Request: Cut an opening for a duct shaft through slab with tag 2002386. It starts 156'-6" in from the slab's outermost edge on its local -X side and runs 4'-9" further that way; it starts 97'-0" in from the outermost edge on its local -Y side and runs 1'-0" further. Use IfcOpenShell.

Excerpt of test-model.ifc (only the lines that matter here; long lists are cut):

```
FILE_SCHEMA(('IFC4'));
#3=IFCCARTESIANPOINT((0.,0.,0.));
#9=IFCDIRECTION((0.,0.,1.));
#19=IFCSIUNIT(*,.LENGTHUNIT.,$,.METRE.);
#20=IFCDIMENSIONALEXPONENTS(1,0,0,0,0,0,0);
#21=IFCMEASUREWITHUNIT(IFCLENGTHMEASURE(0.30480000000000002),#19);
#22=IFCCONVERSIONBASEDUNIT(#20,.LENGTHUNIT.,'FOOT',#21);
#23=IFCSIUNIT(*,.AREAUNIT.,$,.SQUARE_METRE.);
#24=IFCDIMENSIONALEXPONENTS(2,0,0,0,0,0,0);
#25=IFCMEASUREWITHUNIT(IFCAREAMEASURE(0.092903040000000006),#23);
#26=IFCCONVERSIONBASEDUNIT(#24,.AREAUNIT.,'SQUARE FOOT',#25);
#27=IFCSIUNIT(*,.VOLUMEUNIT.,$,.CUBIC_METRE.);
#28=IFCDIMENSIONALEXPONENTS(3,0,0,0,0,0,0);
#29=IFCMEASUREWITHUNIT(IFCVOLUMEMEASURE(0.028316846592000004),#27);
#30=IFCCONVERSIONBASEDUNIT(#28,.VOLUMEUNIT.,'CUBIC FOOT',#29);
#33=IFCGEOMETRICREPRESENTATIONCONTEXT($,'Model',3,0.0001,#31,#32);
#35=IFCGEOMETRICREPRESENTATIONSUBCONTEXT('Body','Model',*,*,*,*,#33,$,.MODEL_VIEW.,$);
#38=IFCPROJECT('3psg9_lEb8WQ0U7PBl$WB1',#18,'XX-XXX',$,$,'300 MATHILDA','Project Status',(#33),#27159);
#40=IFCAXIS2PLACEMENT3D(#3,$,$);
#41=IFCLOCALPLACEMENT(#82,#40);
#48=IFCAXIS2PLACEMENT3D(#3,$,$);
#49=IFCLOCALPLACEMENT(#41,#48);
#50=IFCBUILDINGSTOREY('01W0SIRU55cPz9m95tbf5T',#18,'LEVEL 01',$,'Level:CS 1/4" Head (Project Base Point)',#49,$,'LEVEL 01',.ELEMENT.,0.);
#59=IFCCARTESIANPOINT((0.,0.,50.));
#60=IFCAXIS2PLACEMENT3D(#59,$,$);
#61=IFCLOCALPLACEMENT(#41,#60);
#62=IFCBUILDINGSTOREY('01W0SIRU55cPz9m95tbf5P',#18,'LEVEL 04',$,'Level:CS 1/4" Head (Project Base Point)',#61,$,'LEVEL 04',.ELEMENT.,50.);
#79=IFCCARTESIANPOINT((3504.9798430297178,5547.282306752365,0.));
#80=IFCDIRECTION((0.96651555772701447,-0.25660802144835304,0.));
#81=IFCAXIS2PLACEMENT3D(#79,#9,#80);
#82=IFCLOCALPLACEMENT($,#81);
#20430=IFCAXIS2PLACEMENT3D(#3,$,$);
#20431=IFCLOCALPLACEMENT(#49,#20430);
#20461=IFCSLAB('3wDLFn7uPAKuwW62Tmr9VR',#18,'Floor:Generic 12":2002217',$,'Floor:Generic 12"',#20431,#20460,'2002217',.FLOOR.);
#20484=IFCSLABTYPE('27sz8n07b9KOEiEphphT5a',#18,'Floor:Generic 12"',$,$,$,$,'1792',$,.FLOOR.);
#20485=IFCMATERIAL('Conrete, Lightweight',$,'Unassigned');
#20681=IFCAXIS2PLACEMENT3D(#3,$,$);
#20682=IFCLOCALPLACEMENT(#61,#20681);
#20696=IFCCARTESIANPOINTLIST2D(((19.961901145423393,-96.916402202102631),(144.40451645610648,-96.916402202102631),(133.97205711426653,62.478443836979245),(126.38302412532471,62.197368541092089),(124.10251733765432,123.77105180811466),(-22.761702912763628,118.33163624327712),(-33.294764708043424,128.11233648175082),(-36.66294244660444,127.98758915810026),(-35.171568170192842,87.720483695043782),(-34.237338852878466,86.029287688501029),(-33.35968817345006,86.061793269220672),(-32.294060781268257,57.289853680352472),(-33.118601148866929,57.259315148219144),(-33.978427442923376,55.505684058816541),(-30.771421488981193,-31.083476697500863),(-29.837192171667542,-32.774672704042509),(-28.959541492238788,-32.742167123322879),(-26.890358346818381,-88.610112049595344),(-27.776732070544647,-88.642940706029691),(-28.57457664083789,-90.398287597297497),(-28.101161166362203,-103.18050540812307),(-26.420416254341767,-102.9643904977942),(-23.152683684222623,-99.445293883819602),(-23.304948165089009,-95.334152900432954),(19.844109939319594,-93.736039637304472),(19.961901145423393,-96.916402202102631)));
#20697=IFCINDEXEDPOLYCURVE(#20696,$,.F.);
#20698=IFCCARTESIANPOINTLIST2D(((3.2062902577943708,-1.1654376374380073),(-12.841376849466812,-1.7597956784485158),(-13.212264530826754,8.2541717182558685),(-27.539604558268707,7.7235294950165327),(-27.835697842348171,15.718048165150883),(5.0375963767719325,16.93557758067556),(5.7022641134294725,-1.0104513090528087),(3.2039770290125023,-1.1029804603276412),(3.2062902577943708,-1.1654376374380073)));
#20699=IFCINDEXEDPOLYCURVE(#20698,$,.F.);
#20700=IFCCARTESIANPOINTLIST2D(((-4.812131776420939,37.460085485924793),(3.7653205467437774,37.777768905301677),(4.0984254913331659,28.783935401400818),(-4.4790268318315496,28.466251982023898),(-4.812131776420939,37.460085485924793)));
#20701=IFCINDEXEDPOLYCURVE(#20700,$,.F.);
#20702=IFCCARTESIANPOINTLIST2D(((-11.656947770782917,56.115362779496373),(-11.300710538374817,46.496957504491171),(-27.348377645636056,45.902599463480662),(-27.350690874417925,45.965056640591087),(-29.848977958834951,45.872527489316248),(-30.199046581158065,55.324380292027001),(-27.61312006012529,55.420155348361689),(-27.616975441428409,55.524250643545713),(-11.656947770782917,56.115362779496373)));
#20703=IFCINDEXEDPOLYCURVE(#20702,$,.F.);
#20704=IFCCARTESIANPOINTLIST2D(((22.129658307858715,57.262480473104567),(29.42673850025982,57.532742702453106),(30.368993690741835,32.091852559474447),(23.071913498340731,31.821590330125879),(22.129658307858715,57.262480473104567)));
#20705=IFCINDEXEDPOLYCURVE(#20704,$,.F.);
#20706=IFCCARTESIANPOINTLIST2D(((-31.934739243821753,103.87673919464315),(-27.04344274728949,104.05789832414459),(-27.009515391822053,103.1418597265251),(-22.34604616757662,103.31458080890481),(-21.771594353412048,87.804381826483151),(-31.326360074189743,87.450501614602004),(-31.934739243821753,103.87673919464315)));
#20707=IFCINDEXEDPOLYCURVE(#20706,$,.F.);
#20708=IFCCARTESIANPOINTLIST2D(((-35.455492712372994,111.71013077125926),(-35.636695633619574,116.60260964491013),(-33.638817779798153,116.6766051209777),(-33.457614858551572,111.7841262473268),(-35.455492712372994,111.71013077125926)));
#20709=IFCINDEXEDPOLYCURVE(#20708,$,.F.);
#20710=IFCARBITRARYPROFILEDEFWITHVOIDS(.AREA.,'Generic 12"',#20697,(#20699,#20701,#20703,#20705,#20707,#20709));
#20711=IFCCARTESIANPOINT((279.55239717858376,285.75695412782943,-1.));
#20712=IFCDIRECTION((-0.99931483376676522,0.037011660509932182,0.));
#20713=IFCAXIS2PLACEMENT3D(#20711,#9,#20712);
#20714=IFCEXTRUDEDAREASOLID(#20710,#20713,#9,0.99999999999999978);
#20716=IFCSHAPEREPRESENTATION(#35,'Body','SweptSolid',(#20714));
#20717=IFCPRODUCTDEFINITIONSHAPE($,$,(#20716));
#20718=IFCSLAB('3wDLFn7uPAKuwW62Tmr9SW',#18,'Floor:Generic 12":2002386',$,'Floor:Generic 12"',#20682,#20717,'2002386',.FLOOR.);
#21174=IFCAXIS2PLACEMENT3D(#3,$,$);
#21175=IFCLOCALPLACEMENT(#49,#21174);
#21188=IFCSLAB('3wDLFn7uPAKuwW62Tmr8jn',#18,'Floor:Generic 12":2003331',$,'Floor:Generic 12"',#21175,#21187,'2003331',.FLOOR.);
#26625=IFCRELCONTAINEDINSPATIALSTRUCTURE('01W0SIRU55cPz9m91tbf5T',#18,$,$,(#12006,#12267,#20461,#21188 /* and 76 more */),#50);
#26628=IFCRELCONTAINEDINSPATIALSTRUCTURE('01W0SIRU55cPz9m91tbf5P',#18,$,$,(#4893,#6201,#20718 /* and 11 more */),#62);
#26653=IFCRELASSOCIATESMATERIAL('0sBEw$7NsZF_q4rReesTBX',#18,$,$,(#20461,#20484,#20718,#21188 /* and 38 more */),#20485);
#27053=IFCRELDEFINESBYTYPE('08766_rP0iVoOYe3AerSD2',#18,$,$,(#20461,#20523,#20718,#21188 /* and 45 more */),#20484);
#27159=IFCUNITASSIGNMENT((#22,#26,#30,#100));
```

```python
import numpy as np
import ifcopenshell
import ifcopenshell.api.feature
import ifcopenshell.api.geometry
import ifcopenshell.api.root
import ifcopenshell.geom
import ifcopenshell.util.placement
import ifcopenshell.util.representation
import ifcopenshell.util.shape
import ifcopenshell.util.unit

model = ifcopenshell.open("test-model.ifc")
unit_scale = ifcopenshell.util.unit.calculate_unit_scale(model)
settings = ifcopenshell.geom.settings()


def volume(element):
    """Net volume in cubic metres, openings subtracted."""
    shape = ifcopenshell.geom.create_shape(settings, element)
    return ifcopenshell.util.shape.get_volume(shape.geometry)


slab = model.by_guid("3wDLFn7uPAKuwW62Tmr9SW")
before = volume(slab)

# Extent in the slab's own axes, in metres. The edges named are its -X and -Y sides.
slab_shape = ifcopenshell.geom.create_shape(settings, slab)
vertices = ifcopenshell.util.shape.get_vertices(slab_shape.geometry)
x_min, y_min, bottom = vertices.min(axis=0)
top = vertices[:, 2].max()

opening = ifcopenshell.api.root.create_entity(model, ifc_class="IfcOpeningElement", name="Duct shaft opening", predefined_type="OPENING")
context = ifcopenshell.util.representation.get_context(model, "Model", "Body", "MODEL_VIEW")
width, depth = 1.4478, 0.3048
outline = [(0.0, 0.0), (width, 0.0), (width, depth), (0.0, depth), (0.0, 0.0)]
# Overshoot both faces by 50 mm so the cut is clean.
shape = ifcopenshell.api.geometry.add_slab_representation(
    model, context=context, depth=top - bottom + 0.1, polyline=outline
)
ifcopenshell.api.geometry.assign_representation(model, product=opening, representation=shape)

matrix = ifcopenshell.util.placement.get_local_placement(slab.ObjectPlacement)
matrix[:, 3] = matrix @ np.append(np.array([x_min + 47.7012, y_min + 29.5656, bottom - 0.05]) / unit_scale, 1.0)
ifcopenshell.api.geometry.edit_object_placement(model, product=opening, matrix=matrix, is_si=False)
ifcopenshell.api.feature.add_feature(model, feature=opening, element=slab)

after = volume(slab)

print(f"slab volume {before:.3f} -> {after:.3f} m3")

model.write("test-model_rev.ifc")
```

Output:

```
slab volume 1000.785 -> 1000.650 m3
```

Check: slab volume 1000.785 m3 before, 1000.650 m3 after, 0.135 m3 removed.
